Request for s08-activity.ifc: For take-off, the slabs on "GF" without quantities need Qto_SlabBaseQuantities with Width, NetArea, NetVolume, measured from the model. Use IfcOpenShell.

First a look at what the model holds.

```python
import ifcopenshell
import ifcopenshell.util.element
import ifcopenshell.util.unit

model = ifcopenshell.open("s08-activity.ifc")
print(model.schema)
for unit_type in ("LENGTHUNIT", "AREAUNIT", "VOLUMEUNIT"):
    print(unit_type, ifcopenshell.util.unit.calculate_unit_scale(model, unit_type))
storey = next(s for s in model.by_type("IfcBuildingStorey") if s.Name == "GF")
slabs = [e for e in ifcopenshell.util.element.get_decomposition(storey) if e.is_a("IfcSlab")]
for e in sorted(slabs, key=lambda e: e.id()):
    print(e.id(), e.is_a(), e.Name, list(ifcopenshell.util.element.get_psets(e, qtos_only=True)), sep=" | ")
```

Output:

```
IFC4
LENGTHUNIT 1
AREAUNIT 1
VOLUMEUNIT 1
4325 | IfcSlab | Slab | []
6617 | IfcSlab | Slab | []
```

```python
import ifcopenshell
import ifcopenshell.api.pset
import ifcopenshell.geom
import ifcopenshell.util.element
import ifcopenshell.util.shape
import ifcopenshell.util.unit

model = ifcopenshell.open("s08-activity.ifc")
unit_scale = ifcopenshell.util.unit.calculate_unit_scale(model)
area_scale = ifcopenshell.util.unit.calculate_unit_scale(model, "AREAUNIT")
volume_scale = ifcopenshell.util.unit.calculate_unit_scale(model, "VOLUMEUNIT")
settings = ifcopenshell.geom.settings()

storey = next(s for s in model.by_type("IfcBuildingStorey") if s.Name == "GF")
slabs = [e for e in ifcopenshell.util.element.get_decomposition(storey) if e.is_a("IfcSlab")]

for e in sorted(slabs, key=lambda e: e.id()):
    if ifcopenshell.util.element.get_psets(e, qtos_only=True, should_inherit=False):
        continue
    # Geometry comes back in metres, in the element's own axes.
    shape = ifcopenshell.geom.create_shape(settings, e)
    values = {
        "Width": ifcopenshell.util.shape.get_z(shape.geometry) / unit_scale,
        "NetArea": ifcopenshell.util.shape.get_footprint_area(shape.geometry) / area_scale,
        "NetVolume": ifcopenshell.util.shape.get_volume(shape.geometry) / volume_scale,
    }
    qto = ifcopenshell.api.pset.add_qto(model, product=e, name="Qto_SlabBaseQuantities")
    ifcopenshell.api.pset.edit_qto(model, qto=qto, properties=values)
    print(e.id(), {k: round(v, 3) for k, v in values.items()})

model.write("s08-activity-out.ifc")
```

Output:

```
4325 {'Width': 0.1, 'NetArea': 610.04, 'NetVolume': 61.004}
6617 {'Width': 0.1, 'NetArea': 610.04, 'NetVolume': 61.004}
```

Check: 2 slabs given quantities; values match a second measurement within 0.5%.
